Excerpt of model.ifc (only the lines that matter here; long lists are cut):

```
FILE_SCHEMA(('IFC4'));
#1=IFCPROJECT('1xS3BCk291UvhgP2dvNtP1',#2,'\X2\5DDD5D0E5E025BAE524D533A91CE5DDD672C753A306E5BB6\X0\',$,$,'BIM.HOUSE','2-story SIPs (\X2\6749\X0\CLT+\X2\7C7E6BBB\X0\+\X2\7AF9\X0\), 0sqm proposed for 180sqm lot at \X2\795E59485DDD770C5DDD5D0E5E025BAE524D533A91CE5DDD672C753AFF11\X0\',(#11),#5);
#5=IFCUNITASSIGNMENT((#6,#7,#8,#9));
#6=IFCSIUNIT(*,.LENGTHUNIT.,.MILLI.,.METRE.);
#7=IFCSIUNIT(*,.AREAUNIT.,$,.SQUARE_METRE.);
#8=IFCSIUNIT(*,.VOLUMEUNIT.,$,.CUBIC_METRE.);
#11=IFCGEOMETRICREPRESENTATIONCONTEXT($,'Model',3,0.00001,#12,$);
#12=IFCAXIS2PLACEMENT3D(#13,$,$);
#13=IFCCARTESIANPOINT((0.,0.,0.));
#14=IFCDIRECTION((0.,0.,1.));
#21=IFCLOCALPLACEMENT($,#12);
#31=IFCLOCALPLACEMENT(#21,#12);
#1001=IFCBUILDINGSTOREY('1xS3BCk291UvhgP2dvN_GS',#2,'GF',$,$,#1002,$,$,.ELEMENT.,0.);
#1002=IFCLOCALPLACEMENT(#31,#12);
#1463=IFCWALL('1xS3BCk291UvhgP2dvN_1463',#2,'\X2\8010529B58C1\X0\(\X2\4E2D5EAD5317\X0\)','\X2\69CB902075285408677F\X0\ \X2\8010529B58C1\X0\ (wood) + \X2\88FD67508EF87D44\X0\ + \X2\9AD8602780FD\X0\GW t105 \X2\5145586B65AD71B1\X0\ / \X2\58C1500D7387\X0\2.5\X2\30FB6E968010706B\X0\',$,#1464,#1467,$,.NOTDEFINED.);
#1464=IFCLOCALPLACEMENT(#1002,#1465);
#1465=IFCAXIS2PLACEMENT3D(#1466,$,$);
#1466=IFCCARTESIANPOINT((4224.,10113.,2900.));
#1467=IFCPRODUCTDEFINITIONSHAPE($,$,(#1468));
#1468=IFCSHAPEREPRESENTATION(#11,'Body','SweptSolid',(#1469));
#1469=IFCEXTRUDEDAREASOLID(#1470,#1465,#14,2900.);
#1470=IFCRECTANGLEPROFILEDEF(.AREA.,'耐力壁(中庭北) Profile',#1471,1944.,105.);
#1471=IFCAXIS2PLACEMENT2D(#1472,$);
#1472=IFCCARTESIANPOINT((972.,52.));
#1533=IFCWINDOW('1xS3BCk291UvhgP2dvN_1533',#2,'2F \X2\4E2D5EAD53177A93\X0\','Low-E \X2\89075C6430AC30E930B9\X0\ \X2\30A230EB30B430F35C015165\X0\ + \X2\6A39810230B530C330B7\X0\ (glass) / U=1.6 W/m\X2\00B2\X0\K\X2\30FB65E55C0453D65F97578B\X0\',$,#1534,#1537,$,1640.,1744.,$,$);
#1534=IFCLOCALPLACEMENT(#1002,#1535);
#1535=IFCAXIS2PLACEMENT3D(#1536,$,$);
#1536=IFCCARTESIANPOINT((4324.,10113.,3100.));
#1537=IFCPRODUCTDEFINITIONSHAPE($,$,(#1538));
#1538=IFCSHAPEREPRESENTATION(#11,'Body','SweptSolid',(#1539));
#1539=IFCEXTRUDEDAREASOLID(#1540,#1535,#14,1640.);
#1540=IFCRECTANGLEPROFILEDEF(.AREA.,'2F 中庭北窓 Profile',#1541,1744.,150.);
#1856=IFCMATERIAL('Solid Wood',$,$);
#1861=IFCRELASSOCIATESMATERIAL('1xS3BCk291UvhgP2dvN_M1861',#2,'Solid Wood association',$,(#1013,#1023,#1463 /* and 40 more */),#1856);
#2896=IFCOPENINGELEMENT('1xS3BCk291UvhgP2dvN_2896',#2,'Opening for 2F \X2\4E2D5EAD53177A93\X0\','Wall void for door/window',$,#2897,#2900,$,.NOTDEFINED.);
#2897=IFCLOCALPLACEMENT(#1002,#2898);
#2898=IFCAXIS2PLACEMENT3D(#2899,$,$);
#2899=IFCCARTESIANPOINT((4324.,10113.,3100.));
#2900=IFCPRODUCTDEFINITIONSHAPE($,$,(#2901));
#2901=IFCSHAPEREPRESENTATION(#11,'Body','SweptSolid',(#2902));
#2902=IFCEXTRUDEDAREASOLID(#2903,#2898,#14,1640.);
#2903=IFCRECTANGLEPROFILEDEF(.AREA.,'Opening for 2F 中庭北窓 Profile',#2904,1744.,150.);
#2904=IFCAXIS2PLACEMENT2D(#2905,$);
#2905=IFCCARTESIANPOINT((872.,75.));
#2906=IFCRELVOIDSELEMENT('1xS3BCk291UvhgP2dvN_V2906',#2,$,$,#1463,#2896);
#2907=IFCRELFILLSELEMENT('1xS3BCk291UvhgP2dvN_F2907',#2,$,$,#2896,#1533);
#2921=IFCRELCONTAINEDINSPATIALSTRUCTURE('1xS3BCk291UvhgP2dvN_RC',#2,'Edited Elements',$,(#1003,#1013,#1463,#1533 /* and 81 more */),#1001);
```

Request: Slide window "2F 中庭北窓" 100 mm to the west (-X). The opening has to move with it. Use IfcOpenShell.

```python
import ifcopenshell
import ifcopenshell.api.geometry
import ifcopenshell.util.placement
import ifcopenshell.util.unit

model = ifcopenshell.open("model.ifc")
unit_scale = ifcopenshell.util.unit.calculate_unit_scale(model)

window = model.by_guid("1xS3BCk291UvhgP2dvN_1533")
opening = window.FillsVoids[0].RelatingOpeningElement
wall = opening.VoidsElements[0].RelatingBuildingElement

wall_matrix = ifcopenshell.util.placement.get_local_placement(wall.ObjectPlacement)
shift = wall_matrix[:3, 0] * -0.1 / unit_scale
before = ifcopenshell.util.placement.get_local_placement(window.ObjectPlacement)[:3, 3].copy()

# The window is not placed relative to its opening, so move both.
for product in (opening, window):
    matrix = ifcopenshell.util.placement.get_local_placement(product.ObjectPlacement)
    matrix[:3, 3] += shift
    ifcopenshell.api.geometry.edit_object_placement(model, product=product, matrix=matrix, is_si=False)

after = ifcopenshell.util.placement.get_local_placement(window.ObjectPlacement)[:3, 3]
print("window moved by", (after - before).round(3) + 0.0)

model.write("model_v2.ifc")
```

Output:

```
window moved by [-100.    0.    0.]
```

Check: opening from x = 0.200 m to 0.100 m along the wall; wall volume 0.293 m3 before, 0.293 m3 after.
